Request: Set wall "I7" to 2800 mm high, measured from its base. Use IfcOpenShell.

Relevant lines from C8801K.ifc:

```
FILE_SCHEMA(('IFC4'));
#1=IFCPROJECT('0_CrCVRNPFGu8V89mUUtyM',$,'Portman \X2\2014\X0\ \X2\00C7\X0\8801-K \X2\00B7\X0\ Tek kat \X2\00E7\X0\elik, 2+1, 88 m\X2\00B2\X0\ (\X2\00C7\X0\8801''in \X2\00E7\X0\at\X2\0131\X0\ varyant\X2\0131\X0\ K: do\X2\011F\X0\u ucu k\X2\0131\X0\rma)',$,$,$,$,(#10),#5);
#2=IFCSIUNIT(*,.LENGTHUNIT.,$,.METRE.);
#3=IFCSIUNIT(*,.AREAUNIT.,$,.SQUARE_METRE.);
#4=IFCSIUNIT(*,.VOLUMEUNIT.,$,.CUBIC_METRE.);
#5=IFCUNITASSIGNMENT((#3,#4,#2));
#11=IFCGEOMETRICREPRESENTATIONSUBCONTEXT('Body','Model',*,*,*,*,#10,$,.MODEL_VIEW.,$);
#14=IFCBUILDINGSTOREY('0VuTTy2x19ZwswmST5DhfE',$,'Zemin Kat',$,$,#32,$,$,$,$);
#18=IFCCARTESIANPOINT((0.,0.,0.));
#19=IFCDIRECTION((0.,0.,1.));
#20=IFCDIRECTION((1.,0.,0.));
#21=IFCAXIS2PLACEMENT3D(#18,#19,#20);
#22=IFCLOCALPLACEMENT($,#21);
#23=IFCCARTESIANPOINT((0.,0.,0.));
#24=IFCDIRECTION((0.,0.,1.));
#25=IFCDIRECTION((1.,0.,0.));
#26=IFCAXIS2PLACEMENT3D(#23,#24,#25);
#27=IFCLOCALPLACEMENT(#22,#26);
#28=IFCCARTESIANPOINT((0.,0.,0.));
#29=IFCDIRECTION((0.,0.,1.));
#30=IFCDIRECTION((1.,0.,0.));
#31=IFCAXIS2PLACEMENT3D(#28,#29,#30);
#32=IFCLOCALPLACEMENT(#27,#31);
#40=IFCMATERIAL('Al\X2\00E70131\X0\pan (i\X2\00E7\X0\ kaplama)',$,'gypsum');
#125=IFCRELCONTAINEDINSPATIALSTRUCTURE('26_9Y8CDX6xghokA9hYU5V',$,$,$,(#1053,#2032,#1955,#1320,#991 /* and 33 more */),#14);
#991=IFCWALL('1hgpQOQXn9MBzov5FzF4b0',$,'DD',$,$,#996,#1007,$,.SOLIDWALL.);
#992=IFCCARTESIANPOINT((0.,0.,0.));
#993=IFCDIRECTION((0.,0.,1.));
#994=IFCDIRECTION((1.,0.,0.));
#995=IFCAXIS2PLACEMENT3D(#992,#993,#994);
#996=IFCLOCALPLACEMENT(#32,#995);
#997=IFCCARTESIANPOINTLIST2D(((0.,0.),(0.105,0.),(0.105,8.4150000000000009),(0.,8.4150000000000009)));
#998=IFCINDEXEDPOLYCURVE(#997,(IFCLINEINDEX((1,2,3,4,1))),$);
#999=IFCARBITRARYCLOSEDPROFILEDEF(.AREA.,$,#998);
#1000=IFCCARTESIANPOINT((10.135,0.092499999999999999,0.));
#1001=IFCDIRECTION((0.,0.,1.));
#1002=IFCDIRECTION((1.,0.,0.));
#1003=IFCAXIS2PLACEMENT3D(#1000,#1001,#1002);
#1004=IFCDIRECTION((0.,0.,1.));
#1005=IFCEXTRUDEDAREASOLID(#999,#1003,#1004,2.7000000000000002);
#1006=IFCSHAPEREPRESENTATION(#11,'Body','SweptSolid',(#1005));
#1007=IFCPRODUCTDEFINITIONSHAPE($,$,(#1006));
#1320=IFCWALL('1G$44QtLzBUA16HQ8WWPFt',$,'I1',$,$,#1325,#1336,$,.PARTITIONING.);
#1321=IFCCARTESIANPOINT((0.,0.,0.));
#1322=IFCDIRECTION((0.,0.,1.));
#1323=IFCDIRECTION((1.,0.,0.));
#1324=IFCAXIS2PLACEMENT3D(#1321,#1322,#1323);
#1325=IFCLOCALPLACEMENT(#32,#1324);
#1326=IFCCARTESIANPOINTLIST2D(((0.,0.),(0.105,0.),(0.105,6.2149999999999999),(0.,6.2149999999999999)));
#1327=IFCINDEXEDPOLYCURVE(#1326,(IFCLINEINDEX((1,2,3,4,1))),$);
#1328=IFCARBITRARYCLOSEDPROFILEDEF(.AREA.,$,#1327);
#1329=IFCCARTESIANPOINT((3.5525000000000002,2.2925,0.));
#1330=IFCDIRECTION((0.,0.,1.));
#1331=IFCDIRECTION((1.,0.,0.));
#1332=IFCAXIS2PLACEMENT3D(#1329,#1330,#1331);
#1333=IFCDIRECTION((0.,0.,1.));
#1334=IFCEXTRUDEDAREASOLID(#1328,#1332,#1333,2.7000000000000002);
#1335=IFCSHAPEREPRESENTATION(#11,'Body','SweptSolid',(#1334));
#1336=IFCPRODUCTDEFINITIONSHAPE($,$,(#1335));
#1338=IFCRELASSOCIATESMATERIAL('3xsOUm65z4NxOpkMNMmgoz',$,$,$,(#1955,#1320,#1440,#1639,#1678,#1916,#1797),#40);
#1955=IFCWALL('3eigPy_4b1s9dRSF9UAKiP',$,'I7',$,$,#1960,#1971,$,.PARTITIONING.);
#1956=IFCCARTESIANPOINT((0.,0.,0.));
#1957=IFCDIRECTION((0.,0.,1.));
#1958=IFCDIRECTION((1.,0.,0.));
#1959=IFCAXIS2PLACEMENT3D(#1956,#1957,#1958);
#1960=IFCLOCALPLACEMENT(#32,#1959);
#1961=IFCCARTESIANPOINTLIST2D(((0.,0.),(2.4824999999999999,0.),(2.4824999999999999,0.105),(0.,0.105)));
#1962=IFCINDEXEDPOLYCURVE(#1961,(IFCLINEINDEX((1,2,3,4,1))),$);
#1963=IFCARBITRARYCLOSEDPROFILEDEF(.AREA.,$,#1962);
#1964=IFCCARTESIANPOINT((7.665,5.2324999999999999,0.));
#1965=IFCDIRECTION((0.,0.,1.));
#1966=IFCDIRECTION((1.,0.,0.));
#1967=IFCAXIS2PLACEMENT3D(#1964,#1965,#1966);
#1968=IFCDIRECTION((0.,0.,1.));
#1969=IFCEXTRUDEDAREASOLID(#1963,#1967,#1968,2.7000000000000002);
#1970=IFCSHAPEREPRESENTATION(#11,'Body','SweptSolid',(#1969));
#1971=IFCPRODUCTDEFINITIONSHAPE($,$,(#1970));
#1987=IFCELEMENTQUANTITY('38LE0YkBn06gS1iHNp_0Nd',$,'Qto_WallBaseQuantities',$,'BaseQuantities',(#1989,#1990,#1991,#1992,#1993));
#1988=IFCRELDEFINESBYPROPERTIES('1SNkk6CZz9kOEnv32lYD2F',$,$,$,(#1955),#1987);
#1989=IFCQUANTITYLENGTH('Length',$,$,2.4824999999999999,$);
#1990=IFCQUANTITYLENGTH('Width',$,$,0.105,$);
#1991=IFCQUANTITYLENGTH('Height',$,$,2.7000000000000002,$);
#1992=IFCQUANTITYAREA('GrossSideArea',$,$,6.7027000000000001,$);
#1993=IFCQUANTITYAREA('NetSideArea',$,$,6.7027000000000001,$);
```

```python
import ifcopenshell
import ifcopenshell.api.pset
import ifcopenshell.geom
import ifcopenshell.util.element
import ifcopenshell.util.representation
import ifcopenshell.util.shape
import ifcopenshell.util.unit

model = ifcopenshell.open("C8801K.ifc")
unit_scale = ifcopenshell.util.unit.calculate_unit_scale(model)
area_scale = ifcopenshell.util.unit.calculate_unit_scale(model, "AREAUNIT")
settings = ifcopenshell.geom.settings()


def volume(element):
    """Net volume in cubic metres, openings subtracted."""
    shape = ifcopenshell.geom.create_shape(settings, element)
    return ifcopenshell.util.shape.get_volume(shape.geometry)


wall = model.by_guid("3eigPy_4b1s9dRSF9UAKiP")
before = volume(wall)

body = ifcopenshell.util.representation.get_representation(wall, "Model", "Body")
solid = body.Items[0]
old_height = solid.Depth
solid.Depth = 2.8
after = volume(wall)
thickness = 0.105  # wall thickness in metres

# Update the stored height, areas and volumes.
qto = model.by_id(ifcopenshell.util.element.get_pset(wall, "Qto_WallBaseQuantities", should_inherit=False)["id"])
ifcopenshell.api.pset.edit_qto(model, qto=qto, properties={
    "Height": solid.Depth,
    "GrossSideArea": ifcopenshell.util.element.get_pset(wall, "Qto_WallBaseQuantities", "GrossSideArea") * solid.Depth / old_height,
    "NetSideArea": after / thickness / area_scale,
})

print(f"height {old_height:g} -> {solid.Depth:g}, volume {before:.3f} -> {after:.3f} m3")

model.write("C8801K_edited.ifc")
```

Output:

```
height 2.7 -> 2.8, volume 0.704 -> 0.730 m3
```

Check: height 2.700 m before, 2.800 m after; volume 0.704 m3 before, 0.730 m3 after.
